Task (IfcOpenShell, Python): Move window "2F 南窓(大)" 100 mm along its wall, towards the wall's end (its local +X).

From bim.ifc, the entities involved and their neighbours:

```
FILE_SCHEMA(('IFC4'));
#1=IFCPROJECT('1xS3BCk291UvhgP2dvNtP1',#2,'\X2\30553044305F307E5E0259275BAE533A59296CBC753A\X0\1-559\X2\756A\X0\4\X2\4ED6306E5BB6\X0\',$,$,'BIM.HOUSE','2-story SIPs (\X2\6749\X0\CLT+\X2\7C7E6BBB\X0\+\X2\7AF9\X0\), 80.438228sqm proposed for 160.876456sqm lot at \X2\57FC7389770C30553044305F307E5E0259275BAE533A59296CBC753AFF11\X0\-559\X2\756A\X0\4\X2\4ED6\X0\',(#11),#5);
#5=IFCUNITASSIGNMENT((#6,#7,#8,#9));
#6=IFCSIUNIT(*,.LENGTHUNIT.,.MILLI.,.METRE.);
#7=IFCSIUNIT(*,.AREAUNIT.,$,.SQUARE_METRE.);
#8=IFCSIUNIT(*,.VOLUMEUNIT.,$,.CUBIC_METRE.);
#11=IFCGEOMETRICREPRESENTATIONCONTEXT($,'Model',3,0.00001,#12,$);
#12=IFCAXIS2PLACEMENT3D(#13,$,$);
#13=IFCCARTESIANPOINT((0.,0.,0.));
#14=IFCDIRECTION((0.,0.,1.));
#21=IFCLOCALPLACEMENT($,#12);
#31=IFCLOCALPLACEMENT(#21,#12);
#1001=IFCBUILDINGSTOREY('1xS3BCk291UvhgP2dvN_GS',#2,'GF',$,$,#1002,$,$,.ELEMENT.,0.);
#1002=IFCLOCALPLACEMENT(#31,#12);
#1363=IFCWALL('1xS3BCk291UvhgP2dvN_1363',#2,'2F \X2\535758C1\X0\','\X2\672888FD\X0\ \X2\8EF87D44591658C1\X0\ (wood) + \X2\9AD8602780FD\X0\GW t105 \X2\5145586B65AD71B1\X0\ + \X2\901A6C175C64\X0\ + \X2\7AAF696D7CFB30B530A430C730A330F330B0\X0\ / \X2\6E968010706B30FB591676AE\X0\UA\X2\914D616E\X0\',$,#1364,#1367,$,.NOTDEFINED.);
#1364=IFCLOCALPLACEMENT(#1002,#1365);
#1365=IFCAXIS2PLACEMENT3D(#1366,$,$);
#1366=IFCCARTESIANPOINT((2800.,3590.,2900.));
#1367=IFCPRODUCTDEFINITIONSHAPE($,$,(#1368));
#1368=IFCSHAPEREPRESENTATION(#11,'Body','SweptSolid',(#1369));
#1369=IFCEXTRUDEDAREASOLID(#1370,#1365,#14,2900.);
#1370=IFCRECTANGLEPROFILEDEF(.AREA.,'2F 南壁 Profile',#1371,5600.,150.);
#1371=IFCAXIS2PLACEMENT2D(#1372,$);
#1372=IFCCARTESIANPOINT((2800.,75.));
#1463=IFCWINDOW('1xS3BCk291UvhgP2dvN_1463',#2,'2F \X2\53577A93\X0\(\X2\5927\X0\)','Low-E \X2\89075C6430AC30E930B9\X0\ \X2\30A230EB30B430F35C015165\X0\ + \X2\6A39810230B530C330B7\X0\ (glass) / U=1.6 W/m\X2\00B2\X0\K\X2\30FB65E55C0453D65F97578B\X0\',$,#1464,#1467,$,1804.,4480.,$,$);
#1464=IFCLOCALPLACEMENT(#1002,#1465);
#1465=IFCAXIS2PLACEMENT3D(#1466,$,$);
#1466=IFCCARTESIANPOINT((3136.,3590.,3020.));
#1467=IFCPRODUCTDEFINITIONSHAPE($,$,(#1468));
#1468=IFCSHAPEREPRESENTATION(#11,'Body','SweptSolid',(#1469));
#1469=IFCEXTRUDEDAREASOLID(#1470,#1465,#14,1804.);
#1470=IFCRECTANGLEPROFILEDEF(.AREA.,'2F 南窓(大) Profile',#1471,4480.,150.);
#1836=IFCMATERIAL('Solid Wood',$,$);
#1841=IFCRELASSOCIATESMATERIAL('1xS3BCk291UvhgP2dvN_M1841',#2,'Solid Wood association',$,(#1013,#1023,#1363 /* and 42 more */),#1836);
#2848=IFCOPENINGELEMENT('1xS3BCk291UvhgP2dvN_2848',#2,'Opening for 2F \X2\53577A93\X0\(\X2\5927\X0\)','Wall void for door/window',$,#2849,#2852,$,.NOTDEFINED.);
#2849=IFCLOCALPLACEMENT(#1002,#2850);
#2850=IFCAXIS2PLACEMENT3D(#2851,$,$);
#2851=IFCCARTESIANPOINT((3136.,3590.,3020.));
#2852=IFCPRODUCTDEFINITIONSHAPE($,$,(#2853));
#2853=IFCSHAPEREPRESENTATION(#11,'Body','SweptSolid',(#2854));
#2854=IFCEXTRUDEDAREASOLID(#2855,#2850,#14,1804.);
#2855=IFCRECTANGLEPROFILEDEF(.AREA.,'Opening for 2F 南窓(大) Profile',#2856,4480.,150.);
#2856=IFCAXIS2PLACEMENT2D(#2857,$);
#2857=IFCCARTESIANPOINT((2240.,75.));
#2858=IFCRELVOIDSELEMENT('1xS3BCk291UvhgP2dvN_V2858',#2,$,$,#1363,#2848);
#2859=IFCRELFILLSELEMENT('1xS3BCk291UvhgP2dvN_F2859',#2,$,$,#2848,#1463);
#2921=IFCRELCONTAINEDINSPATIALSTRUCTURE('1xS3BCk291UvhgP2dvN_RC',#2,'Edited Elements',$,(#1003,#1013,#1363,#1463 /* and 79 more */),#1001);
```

```python
import ifcopenshell
import ifcopenshell.api.geometry
import ifcopenshell.util.placement

model = ifcopenshell.open("bim.ifc")

window = model.by_guid("1xS3BCk291UvhgP2dvN_1463")
opening = window.FillsVoids[0].RelatingOpeningElement
wall = opening.VoidsElements[0].RelatingBuildingElement

wall_matrix = ifcopenshell.util.placement.get_local_placement(wall.ObjectPlacement)
shift = wall_matrix[:3, 0] * 100.0
before = ifcopenshell.util.placement.get_local_placement(window.ObjectPlacement)[:3, 3].copy()

# The window is not placed relative to its opening, so move both.
for product in (opening, window):
    matrix = ifcopenshell.util.placement.get_local_placement(product.ObjectPlacement)
    matrix[:3, 3] += shift
    ifcopenshell.api.geometry.edit_object_placement(model, product=product, matrix=matrix, is_si=False)

after = ifcopenshell.util.placement.get_local_placement(window.ObjectPlacement)[:3, 3]
print("window moved by", (after - before).round(3) + 0.0)

model.write("bim_rev.ifc")
```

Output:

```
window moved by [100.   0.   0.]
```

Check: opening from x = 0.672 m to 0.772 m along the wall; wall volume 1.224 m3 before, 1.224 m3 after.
